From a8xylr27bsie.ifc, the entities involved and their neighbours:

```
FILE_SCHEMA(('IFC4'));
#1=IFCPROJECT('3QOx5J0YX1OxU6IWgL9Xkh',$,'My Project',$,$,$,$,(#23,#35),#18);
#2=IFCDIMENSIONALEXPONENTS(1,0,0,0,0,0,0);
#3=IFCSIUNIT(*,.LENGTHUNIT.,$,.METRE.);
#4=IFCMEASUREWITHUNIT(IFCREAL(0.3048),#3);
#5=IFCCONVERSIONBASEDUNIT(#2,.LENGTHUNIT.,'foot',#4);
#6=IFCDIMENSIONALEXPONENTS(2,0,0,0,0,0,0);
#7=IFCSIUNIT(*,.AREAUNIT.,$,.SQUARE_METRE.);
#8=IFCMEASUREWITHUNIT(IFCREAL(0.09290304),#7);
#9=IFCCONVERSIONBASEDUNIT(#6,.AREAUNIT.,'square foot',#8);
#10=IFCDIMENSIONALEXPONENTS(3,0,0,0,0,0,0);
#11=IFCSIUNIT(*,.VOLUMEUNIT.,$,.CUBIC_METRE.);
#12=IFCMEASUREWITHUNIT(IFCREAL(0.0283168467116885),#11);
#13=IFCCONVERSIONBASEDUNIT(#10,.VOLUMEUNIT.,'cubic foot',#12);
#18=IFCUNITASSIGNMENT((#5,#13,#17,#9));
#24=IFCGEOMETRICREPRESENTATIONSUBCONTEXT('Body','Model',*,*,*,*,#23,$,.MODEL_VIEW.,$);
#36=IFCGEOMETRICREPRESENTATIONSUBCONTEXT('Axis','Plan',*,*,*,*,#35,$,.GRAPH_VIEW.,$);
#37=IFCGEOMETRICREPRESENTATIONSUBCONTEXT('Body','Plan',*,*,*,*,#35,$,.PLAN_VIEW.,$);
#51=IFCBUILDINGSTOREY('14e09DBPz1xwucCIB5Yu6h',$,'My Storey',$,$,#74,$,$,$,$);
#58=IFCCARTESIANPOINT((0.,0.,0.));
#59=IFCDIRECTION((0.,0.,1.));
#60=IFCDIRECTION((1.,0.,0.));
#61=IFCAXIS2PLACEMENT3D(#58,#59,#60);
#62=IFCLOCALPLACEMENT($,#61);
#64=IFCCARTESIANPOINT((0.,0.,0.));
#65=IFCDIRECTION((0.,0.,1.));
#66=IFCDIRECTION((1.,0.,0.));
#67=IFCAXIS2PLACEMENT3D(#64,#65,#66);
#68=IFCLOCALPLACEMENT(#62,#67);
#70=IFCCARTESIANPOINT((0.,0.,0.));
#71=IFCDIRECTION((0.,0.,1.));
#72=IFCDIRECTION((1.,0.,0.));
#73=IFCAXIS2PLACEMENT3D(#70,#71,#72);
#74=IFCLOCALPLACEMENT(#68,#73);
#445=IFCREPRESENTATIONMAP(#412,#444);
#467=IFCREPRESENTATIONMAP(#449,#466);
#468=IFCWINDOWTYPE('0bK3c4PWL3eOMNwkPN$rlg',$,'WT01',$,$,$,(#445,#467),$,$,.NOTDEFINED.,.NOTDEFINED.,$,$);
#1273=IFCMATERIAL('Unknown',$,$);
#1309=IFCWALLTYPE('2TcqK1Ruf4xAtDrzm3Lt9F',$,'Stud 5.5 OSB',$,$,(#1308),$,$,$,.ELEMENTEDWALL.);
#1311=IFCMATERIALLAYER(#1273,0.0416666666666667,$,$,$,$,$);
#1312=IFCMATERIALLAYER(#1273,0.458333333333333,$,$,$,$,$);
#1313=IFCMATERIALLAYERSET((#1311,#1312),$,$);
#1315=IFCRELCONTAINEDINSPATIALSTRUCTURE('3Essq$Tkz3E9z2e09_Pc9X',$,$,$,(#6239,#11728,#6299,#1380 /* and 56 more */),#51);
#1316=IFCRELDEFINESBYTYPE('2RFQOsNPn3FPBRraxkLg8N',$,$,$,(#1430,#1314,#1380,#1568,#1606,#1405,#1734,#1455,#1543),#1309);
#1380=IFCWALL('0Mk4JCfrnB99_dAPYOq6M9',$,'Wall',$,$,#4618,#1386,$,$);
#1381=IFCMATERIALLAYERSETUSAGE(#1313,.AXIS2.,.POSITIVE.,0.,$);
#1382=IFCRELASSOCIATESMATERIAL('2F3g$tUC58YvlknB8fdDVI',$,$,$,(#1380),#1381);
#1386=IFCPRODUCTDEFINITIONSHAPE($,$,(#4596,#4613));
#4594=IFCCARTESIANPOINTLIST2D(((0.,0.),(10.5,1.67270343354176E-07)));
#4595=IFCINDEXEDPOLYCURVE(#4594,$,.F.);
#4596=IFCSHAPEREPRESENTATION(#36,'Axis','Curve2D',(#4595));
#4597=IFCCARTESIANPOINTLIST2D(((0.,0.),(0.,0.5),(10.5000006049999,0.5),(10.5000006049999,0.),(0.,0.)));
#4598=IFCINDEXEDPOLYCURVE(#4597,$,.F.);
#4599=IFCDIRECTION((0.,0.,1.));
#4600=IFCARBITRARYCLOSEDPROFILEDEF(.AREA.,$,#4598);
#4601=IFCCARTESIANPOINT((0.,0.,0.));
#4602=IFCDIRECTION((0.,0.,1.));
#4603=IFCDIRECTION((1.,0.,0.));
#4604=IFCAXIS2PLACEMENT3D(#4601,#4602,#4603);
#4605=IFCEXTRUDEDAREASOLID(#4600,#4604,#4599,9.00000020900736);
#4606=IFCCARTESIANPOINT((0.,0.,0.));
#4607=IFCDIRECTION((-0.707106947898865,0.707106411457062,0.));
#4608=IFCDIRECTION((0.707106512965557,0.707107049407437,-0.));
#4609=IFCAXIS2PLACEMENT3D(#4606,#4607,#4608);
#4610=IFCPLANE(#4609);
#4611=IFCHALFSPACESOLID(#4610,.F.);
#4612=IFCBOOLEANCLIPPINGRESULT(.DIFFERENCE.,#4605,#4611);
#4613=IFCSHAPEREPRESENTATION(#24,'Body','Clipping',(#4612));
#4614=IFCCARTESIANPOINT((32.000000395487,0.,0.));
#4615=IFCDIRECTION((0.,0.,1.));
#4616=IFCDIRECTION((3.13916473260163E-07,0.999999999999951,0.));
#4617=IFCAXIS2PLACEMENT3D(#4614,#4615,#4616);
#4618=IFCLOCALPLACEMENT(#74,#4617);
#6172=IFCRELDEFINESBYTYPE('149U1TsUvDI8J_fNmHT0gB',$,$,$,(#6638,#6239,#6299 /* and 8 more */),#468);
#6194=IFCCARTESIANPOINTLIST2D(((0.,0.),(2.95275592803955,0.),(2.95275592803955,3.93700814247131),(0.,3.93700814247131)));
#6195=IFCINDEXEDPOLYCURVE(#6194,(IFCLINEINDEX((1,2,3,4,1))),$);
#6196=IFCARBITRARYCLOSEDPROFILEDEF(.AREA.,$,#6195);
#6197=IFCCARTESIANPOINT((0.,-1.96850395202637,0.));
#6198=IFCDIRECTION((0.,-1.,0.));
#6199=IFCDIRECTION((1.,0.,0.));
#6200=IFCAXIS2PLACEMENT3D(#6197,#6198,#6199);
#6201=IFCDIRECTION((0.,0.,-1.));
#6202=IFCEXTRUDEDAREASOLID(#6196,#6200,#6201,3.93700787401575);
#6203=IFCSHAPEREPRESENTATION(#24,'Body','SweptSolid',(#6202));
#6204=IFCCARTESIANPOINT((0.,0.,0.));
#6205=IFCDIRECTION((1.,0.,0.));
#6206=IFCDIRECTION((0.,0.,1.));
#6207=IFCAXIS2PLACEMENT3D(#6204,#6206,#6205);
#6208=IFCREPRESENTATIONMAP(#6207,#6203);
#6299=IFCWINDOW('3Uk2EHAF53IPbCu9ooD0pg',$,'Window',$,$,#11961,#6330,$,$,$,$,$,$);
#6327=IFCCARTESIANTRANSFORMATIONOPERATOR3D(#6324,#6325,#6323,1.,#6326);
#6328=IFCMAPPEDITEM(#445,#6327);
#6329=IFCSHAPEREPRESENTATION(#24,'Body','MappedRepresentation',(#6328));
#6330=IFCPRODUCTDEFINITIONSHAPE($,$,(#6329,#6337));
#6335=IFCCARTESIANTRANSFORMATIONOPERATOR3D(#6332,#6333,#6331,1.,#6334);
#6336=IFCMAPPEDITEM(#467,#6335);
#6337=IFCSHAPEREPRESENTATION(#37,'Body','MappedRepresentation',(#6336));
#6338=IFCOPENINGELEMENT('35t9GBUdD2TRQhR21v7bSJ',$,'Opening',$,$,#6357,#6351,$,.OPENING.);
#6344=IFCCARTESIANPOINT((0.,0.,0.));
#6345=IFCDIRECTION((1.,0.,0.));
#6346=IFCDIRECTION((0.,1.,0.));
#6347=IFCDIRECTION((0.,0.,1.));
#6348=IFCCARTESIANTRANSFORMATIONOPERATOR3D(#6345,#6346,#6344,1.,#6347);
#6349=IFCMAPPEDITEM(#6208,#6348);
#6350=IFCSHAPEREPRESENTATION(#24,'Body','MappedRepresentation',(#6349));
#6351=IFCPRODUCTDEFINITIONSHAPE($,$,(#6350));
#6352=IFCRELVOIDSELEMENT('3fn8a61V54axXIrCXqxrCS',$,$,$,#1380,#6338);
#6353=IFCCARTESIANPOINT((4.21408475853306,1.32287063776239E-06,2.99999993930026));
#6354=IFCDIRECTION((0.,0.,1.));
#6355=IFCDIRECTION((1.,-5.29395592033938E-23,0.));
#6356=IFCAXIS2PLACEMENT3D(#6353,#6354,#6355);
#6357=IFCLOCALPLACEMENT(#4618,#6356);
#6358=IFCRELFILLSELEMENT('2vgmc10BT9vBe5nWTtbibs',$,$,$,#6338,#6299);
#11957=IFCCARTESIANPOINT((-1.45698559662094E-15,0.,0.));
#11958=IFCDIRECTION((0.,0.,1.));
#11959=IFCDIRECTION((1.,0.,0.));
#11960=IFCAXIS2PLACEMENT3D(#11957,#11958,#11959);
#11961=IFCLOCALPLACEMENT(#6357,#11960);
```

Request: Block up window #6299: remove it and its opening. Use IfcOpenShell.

```python
import ifcopenshell
import ifcopenshell.api.feature
import ifcopenshell.api.root
import ifcopenshell.geom
import ifcopenshell.util.shape

model = ifcopenshell.open("a8xylr27bsie.ifc")
settings = ifcopenshell.geom.settings()


def volume(element):
    """Net volume in cubic metres, openings subtracted."""
    shape = ifcopenshell.geom.create_shape(settings, element)
    return ifcopenshell.util.shape.get_volume(shape.geometry)


window = model.by_guid("3Uk2EHAF53IPbCu9ooD0pg")
opening = window.FillsVoids[0].RelatingOpeningElement
wall = opening.VoidsElements[0].RelatingBuildingElement
before = volume(wall)

ifcopenshell.api.root.remove_product(model, product=window)
ifcopenshell.api.feature.remove_feature(model, feature=opening)

after = volume(wall)

print(f"wall volume {before:.3f} -> {after:.3f} m3")

model.write("a8xylr27bsie-out.ifc")
```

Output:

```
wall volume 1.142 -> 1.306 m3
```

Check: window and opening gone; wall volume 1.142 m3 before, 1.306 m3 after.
